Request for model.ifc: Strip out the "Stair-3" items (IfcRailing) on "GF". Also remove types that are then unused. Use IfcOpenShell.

First a look at what the model holds.

```python
import ifcopenshell
import ifcopenshell.util.element

model = ifcopenshell.open("model.ifc")
print(model.schema)
storey = next(s for s in model.by_type("IfcBuildingStorey") if s.Name == "GF")
railings = [e for e in ifcopenshell.util.element.get_decomposition(storey) if e.is_a("IfcRailing")]
seen = {}
for e in railings:
    element_type = ifcopenshell.util.element.get_type(e)
    name = element_type.Name if element_type not in (None, e) else None
    seen[name] = seen.get(name, 0) + 1
for name, count in sorted(seen.items(), key=str):
    print(count, "x", name)
```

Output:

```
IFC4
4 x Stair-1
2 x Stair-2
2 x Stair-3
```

```python
import ifcopenshell
import ifcopenshell.api.root
import ifcopenshell.util.element

model = ifcopenshell.open("model.ifc")

storey = next(s for s in model.by_type("IfcBuildingStorey") if s.Name == "GF")
railings = [e for e in ifcopenshell.util.element.get_decomposition(storey) if e.is_a("IfcRailing")]
targets = [e for e in railings if (t := ifcopenshell.util.element.get_type(e)) not in (None, e) and t.Name == "Stair-3"]
types = {ifcopenshell.util.element.get_type(e) for e in targets} - {None, *targets}

for e in targets:
    ifcopenshell.api.root.remove_product(model, product=e)
print(len(targets), "removed")

unused = [t for t in types if not ifcopenshell.util.element.get_types(t)]
for t in unused:
    ifcopenshell.api.root.remove_product(model, product=t)
print(len(unused), "unused types removed")

model.write("model-out.ifc")
```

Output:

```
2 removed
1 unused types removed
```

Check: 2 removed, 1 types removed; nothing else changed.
